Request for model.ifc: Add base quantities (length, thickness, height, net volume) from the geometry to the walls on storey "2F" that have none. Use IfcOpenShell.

First a look at what the model holds.

```python
import ifcopenshell
import ifcopenshell.util.element
import ifcopenshell.util.unit

model = ifcopenshell.open("model.ifc")
print(model.schema)
for unit_type in ("LENGTHUNIT", "AREAUNIT", "VOLUMEUNIT"):
    print(unit_type, ifcopenshell.util.unit.calculate_unit_scale(model, unit_type))
storey = next(s for s in model.by_type("IfcBuildingStorey") if s.Name == "2F")
walls = [e for e in ifcopenshell.util.element.get_decomposition(storey) if e.is_a("IfcWall")]
for e in sorted(walls, key=lambda e: e.id()):
    print(e.id(), e.is_a(), e.Name, list(ifcopenshell.util.element.get_psets(e, qtos_only=True)), sep=" | ")
```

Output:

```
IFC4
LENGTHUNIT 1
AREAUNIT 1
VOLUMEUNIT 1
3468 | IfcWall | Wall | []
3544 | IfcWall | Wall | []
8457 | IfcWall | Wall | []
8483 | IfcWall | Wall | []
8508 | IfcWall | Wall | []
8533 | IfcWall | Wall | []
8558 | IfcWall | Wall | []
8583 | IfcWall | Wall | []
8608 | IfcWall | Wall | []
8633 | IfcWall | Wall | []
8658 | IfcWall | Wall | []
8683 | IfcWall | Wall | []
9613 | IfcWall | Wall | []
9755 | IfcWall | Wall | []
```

```python
import ifcopenshell
import ifcopenshell.api.pset
import ifcopenshell.geom
import ifcopenshell.util.element
import ifcopenshell.util.shape
import ifcopenshell.util.unit

model = ifcopenshell.open("model.ifc")
unit_scale = ifcopenshell.util.unit.calculate_unit_scale(model)
volume_scale = ifcopenshell.util.unit.calculate_unit_scale(model, "VOLUMEUNIT")
settings = ifcopenshell.geom.settings()

storey = next(s for s in model.by_type("IfcBuildingStorey") if s.Name == "2F")
walls = [e for e in ifcopenshell.util.element.get_decomposition(storey) if e.is_a("IfcWall")]

for e in sorted(walls, key=lambda e: e.id()):
    if ifcopenshell.util.element.get_psets(e, qtos_only=True, should_inherit=False):
        continue
    # Geometry comes back in metres, in the element's own axes.
    shape = ifcopenshell.geom.create_shape(settings, e)
    values = {
        "Length": ifcopenshell.util.shape.get_x(shape.geometry) / unit_scale,
        "Width": ifcopenshell.util.shape.get_y(shape.geometry) / unit_scale,
        "Height": ifcopenshell.util.shape.get_z(shape.geometry) / unit_scale,
        "NetVolume": ifcopenshell.util.shape.get_volume(shape.geometry) / volume_scale,
    }
    qto = ifcopenshell.api.pset.add_qto(model, product=e, name="Qto_WallBaseQuantities")
    ifcopenshell.api.pset.edit_qto(model, qto=qto, properties=values)
    print(e.id(), {k: round(v, 3) for k, v in values.items()})

model.write("model_edited.ifc")
```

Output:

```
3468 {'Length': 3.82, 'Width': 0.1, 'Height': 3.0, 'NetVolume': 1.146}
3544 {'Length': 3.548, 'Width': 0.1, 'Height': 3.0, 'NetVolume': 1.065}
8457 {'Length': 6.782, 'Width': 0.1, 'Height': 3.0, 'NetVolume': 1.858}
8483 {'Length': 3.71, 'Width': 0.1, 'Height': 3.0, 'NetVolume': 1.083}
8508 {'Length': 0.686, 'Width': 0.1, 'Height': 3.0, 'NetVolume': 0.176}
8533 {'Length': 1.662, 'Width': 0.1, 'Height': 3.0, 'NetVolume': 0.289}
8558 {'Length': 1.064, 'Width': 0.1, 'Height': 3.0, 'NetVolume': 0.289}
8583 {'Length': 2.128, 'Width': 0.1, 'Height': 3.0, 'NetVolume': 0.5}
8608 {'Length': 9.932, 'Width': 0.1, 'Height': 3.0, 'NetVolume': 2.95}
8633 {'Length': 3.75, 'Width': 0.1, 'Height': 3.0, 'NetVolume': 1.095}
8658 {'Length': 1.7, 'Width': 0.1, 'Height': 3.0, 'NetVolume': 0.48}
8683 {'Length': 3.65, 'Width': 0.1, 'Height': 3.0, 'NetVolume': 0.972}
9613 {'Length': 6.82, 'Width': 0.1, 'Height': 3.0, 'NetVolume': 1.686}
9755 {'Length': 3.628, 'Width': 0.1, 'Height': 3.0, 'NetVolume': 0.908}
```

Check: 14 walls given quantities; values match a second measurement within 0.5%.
